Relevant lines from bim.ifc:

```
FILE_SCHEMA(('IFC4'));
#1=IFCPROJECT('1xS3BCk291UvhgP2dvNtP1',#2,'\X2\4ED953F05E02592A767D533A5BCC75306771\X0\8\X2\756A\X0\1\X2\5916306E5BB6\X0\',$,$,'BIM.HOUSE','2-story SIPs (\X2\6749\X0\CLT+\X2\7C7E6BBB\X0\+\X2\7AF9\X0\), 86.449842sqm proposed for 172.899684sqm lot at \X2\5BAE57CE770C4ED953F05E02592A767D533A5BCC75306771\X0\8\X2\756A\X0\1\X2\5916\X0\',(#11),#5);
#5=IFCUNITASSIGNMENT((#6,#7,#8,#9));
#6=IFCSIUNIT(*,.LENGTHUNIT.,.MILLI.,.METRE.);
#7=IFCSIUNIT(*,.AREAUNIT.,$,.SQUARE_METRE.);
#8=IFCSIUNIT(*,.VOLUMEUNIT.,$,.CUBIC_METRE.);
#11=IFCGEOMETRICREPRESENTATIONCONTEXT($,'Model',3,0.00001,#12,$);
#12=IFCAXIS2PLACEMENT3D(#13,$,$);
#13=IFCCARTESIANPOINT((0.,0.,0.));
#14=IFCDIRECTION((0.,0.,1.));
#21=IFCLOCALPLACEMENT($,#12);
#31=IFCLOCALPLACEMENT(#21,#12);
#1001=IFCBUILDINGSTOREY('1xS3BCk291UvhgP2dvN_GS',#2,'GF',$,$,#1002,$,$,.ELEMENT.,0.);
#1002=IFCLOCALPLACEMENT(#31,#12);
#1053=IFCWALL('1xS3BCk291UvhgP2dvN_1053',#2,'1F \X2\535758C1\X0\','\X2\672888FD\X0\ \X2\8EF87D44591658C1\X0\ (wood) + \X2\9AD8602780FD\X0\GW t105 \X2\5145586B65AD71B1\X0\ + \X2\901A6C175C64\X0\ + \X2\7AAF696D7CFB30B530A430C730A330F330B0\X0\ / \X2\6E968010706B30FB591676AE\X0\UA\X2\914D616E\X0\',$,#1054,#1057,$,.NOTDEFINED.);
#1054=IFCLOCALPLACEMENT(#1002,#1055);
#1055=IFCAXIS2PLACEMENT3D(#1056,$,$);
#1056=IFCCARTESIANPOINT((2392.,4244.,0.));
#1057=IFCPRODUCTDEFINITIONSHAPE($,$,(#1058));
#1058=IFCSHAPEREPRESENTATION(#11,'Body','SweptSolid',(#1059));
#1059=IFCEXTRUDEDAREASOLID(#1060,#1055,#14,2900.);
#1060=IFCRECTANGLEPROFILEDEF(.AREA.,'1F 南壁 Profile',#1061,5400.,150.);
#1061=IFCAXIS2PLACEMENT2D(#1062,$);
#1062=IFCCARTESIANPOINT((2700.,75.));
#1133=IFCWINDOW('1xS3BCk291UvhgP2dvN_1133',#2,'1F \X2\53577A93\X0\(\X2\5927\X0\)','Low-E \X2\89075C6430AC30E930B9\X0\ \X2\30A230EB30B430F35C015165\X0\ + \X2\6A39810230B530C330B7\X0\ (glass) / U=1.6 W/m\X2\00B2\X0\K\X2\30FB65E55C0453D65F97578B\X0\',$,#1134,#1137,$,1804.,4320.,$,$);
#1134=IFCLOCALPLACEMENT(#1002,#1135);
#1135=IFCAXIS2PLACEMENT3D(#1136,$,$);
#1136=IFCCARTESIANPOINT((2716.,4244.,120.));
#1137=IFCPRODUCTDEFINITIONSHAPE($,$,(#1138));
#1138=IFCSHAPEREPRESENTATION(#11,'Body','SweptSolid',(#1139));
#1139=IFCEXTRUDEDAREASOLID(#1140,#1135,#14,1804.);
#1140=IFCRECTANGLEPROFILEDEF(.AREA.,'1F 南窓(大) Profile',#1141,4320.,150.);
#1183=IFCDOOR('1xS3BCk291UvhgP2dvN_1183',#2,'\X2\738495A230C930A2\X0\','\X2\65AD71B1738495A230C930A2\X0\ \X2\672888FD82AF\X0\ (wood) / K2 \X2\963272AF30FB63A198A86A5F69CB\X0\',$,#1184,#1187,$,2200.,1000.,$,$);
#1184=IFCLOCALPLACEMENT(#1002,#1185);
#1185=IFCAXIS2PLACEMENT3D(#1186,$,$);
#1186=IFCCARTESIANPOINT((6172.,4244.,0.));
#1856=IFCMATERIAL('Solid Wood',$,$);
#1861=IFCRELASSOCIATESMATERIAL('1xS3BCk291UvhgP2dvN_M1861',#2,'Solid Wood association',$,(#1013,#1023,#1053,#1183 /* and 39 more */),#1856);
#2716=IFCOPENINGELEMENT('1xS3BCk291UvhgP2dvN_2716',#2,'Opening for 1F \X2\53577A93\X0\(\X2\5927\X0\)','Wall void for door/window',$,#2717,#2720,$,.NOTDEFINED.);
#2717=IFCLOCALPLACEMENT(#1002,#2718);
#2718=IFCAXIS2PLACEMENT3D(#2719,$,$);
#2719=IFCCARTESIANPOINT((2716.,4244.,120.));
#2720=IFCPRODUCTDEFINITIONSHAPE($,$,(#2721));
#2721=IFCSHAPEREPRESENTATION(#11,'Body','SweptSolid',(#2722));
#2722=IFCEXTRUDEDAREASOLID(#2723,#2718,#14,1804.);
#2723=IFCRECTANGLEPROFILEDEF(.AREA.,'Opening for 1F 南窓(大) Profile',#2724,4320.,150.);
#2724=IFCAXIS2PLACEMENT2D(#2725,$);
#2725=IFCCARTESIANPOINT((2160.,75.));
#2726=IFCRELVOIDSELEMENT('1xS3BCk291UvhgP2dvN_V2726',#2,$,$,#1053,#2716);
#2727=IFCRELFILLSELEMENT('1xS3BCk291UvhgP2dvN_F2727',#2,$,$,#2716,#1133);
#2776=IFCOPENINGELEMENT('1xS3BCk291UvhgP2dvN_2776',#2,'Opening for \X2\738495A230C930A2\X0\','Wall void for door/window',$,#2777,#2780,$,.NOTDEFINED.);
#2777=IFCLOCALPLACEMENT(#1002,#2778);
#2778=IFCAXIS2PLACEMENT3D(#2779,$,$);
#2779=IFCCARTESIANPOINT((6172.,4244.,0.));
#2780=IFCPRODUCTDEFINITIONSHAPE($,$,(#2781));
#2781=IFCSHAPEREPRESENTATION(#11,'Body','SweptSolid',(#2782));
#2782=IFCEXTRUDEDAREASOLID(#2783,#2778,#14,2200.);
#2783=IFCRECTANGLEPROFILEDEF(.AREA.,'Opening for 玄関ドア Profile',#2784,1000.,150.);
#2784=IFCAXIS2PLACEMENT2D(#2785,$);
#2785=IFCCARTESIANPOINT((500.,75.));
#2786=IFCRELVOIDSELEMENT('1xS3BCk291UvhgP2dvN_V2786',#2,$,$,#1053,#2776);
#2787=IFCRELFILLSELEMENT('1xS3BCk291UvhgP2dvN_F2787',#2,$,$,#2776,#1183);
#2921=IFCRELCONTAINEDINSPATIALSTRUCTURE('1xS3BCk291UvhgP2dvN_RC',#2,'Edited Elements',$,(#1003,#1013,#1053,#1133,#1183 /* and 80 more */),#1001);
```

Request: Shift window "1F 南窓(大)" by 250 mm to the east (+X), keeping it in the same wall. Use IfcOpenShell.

```python
import ifcopenshell
import ifcopenshell.api.geometry
import ifcopenshell.util.placement

model = ifcopenshell.open("bim.ifc")

window = model.by_guid("1xS3BCk291UvhgP2dvN_1133")
opening = window.FillsVoids[0].RelatingOpeningElement
wall = opening.VoidsElements[0].RelatingBuildingElement

wall_matrix = ifcopenshell.util.placement.get_local_placement(wall.ObjectPlacement)
shift = wall_matrix[:3, 0] * 250.0
before = ifcopenshell.util.placement.get_local_placement(window.ObjectPlacement)[:3, 3].copy()

# The window is not placed relative to its opening, so move both.
for product in (opening, window):
    matrix = ifcopenshell.util.placement.get_local_placement(product.ObjectPlacement)
    matrix[:3, 3] += shift
    ifcopenshell.api.geometry.edit_object_placement(model, product=product, matrix=matrix, is_si=False)

after = ifcopenshell.util.placement.get_local_placement(window.ObjectPlacement)[:3, 3]
print("window moved by", (after - before).round(3) + 0.0)

model.write("bim_v2.ifc")
```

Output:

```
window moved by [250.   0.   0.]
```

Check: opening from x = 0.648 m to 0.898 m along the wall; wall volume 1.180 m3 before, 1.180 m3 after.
